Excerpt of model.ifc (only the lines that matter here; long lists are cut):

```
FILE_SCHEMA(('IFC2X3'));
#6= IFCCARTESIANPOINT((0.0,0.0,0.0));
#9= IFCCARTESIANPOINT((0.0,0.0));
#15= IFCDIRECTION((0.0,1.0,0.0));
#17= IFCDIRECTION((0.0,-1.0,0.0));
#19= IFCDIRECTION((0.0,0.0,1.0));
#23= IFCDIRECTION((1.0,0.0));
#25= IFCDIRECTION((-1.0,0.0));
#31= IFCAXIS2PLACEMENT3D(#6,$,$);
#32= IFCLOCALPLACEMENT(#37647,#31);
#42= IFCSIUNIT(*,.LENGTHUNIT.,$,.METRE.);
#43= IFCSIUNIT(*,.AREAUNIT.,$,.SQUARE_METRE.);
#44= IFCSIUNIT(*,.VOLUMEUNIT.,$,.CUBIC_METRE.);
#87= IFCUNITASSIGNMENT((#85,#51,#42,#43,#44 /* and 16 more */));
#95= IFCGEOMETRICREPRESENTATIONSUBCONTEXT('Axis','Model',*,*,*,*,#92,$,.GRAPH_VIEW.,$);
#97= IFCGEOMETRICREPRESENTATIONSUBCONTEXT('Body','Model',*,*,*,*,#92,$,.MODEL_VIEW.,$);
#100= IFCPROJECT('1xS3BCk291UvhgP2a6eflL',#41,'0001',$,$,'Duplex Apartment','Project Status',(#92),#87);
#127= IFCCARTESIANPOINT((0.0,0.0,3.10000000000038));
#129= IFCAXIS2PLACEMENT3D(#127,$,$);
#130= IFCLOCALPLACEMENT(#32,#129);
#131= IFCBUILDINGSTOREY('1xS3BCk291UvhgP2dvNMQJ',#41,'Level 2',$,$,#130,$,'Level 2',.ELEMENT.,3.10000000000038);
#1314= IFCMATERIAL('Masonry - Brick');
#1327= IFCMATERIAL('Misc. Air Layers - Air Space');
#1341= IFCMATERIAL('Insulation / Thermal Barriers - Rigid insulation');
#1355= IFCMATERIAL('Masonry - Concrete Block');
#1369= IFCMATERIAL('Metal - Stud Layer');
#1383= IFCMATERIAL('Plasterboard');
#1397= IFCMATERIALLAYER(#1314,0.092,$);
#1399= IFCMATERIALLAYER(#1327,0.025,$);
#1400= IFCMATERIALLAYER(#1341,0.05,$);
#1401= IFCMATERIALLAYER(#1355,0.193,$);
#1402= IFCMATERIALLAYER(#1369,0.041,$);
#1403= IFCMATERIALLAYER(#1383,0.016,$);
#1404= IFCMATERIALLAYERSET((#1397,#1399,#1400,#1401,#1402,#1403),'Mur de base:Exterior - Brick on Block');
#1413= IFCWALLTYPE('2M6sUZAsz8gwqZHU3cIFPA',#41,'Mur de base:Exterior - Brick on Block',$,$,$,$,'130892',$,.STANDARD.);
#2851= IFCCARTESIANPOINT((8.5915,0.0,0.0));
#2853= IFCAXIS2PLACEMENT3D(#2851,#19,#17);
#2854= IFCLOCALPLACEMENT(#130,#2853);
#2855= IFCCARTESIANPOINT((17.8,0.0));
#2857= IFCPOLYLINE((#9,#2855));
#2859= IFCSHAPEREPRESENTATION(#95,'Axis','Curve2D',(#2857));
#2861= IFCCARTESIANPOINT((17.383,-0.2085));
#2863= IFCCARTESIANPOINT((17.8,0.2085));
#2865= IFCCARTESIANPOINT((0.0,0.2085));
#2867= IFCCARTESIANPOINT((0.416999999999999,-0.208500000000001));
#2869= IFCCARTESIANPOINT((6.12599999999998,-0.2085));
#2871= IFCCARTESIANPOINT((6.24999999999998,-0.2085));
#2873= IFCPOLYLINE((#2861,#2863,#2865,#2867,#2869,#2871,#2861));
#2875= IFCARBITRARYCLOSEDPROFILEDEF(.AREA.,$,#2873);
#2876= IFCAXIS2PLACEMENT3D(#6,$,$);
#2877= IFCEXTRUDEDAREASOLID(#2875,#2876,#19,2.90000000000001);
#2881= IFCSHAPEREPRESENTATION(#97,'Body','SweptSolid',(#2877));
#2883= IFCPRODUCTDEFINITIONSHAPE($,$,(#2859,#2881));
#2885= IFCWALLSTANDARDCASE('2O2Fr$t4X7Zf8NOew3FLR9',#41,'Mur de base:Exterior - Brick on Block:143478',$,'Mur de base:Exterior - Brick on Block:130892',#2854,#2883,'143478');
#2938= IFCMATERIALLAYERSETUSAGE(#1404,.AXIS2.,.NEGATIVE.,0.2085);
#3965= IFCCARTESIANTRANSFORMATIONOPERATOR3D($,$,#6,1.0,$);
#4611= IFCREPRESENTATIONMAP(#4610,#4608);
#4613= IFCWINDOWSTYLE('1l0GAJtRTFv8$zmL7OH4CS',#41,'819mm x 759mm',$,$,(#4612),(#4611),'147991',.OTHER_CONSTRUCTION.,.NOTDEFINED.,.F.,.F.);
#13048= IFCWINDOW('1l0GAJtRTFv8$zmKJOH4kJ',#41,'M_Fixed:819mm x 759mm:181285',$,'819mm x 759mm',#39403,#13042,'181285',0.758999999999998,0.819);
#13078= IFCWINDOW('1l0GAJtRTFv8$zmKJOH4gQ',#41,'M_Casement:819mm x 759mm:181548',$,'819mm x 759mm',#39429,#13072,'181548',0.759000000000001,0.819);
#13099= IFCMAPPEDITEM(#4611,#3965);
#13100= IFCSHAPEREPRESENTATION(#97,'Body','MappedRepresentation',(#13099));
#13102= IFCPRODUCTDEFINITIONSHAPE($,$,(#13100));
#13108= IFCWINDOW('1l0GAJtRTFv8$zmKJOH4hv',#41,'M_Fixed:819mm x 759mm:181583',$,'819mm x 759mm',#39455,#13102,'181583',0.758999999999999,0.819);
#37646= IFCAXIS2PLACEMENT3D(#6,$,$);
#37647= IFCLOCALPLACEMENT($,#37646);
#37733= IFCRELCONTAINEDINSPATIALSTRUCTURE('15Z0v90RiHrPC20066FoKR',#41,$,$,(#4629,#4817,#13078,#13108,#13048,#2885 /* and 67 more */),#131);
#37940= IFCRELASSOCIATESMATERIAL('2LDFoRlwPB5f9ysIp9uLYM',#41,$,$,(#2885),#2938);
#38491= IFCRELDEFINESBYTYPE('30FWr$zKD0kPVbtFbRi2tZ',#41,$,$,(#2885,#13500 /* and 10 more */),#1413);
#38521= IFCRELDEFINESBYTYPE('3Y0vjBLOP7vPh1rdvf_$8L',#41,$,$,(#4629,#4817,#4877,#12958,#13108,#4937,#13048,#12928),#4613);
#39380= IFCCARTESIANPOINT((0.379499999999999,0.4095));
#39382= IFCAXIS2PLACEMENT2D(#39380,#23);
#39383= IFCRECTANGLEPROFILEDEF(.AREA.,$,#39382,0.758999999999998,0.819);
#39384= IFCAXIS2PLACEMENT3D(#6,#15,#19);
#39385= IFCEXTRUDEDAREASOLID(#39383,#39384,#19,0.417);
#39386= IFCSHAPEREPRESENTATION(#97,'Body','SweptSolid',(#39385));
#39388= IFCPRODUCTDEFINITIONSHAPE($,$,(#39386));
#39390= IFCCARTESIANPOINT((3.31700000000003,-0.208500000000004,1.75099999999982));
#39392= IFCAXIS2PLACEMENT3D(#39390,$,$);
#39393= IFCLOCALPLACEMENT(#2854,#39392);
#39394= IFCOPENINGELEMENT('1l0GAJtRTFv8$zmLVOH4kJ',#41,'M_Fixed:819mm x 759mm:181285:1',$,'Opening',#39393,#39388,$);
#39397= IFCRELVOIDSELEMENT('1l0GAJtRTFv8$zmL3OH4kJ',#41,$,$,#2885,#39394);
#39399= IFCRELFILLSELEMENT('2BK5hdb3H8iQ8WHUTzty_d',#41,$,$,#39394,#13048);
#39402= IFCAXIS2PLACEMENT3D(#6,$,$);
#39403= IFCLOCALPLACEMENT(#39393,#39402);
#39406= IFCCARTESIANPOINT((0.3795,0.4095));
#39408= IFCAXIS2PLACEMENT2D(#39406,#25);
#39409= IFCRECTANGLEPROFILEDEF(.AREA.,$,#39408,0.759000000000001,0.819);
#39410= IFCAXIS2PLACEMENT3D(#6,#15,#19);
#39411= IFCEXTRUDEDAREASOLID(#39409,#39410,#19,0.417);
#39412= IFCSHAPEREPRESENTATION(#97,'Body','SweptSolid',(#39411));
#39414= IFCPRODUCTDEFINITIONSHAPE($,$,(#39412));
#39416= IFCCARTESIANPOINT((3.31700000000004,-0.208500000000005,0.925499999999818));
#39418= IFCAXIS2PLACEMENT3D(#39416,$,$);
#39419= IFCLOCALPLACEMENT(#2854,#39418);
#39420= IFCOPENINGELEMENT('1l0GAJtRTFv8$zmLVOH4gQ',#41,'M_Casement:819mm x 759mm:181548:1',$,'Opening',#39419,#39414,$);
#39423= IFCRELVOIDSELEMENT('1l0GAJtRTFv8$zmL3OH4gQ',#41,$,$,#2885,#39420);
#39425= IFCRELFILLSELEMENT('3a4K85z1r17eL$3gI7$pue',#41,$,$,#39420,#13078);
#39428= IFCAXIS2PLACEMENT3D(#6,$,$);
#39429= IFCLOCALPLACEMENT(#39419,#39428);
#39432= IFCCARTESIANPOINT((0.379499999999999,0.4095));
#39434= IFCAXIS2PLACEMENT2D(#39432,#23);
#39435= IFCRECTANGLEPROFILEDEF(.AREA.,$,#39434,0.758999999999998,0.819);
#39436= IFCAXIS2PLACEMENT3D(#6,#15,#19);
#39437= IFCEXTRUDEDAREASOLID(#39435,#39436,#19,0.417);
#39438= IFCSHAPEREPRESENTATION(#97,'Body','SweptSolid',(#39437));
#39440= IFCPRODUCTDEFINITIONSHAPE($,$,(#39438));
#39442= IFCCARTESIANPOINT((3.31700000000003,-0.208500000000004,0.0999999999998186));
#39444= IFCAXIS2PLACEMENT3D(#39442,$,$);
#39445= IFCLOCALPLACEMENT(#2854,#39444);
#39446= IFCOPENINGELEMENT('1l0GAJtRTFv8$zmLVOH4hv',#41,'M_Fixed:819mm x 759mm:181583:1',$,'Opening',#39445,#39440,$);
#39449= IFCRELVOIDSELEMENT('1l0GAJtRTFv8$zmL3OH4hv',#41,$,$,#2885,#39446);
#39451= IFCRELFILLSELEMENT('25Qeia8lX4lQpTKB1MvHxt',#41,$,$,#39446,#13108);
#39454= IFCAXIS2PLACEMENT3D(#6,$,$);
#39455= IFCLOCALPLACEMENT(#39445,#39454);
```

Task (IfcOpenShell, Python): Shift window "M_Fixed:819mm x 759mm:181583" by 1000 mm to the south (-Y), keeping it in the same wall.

```python
import ifcopenshell
import ifcopenshell.api.geometry
import ifcopenshell.util.placement

model = ifcopenshell.open("model.ifc")

window = model.by_guid("1l0GAJtRTFv8$zmKJOH4hv")
opening = window.FillsVoids[0].RelatingOpeningElement
wall = opening.VoidsElements[0].RelatingBuildingElement

wall_matrix = ifcopenshell.util.placement.get_local_placement(wall.ObjectPlacement)
shift = wall_matrix[:3, 0] * 1.0
before = ifcopenshell.util.placement.get_local_placement(window.ObjectPlacement)[:3, 3].copy()

# The window is placed relative to its opening, so it follows when the opening moves.
matrix = ifcopenshell.util.placement.get_local_placement(opening.ObjectPlacement)
matrix[:3, 3] += shift
ifcopenshell.api.geometry.edit_object_placement(
    model, product=opening, matrix=matrix, is_si=False, should_transform_children=True
)

after = ifcopenshell.util.placement.get_local_placement(window.ObjectPlacement)[:3, 3]
print("window moved by", (after - before).round(3) + 0.0)

model.write("model_rev.ifc")
```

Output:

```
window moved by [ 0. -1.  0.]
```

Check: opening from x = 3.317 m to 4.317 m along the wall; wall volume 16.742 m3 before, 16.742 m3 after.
